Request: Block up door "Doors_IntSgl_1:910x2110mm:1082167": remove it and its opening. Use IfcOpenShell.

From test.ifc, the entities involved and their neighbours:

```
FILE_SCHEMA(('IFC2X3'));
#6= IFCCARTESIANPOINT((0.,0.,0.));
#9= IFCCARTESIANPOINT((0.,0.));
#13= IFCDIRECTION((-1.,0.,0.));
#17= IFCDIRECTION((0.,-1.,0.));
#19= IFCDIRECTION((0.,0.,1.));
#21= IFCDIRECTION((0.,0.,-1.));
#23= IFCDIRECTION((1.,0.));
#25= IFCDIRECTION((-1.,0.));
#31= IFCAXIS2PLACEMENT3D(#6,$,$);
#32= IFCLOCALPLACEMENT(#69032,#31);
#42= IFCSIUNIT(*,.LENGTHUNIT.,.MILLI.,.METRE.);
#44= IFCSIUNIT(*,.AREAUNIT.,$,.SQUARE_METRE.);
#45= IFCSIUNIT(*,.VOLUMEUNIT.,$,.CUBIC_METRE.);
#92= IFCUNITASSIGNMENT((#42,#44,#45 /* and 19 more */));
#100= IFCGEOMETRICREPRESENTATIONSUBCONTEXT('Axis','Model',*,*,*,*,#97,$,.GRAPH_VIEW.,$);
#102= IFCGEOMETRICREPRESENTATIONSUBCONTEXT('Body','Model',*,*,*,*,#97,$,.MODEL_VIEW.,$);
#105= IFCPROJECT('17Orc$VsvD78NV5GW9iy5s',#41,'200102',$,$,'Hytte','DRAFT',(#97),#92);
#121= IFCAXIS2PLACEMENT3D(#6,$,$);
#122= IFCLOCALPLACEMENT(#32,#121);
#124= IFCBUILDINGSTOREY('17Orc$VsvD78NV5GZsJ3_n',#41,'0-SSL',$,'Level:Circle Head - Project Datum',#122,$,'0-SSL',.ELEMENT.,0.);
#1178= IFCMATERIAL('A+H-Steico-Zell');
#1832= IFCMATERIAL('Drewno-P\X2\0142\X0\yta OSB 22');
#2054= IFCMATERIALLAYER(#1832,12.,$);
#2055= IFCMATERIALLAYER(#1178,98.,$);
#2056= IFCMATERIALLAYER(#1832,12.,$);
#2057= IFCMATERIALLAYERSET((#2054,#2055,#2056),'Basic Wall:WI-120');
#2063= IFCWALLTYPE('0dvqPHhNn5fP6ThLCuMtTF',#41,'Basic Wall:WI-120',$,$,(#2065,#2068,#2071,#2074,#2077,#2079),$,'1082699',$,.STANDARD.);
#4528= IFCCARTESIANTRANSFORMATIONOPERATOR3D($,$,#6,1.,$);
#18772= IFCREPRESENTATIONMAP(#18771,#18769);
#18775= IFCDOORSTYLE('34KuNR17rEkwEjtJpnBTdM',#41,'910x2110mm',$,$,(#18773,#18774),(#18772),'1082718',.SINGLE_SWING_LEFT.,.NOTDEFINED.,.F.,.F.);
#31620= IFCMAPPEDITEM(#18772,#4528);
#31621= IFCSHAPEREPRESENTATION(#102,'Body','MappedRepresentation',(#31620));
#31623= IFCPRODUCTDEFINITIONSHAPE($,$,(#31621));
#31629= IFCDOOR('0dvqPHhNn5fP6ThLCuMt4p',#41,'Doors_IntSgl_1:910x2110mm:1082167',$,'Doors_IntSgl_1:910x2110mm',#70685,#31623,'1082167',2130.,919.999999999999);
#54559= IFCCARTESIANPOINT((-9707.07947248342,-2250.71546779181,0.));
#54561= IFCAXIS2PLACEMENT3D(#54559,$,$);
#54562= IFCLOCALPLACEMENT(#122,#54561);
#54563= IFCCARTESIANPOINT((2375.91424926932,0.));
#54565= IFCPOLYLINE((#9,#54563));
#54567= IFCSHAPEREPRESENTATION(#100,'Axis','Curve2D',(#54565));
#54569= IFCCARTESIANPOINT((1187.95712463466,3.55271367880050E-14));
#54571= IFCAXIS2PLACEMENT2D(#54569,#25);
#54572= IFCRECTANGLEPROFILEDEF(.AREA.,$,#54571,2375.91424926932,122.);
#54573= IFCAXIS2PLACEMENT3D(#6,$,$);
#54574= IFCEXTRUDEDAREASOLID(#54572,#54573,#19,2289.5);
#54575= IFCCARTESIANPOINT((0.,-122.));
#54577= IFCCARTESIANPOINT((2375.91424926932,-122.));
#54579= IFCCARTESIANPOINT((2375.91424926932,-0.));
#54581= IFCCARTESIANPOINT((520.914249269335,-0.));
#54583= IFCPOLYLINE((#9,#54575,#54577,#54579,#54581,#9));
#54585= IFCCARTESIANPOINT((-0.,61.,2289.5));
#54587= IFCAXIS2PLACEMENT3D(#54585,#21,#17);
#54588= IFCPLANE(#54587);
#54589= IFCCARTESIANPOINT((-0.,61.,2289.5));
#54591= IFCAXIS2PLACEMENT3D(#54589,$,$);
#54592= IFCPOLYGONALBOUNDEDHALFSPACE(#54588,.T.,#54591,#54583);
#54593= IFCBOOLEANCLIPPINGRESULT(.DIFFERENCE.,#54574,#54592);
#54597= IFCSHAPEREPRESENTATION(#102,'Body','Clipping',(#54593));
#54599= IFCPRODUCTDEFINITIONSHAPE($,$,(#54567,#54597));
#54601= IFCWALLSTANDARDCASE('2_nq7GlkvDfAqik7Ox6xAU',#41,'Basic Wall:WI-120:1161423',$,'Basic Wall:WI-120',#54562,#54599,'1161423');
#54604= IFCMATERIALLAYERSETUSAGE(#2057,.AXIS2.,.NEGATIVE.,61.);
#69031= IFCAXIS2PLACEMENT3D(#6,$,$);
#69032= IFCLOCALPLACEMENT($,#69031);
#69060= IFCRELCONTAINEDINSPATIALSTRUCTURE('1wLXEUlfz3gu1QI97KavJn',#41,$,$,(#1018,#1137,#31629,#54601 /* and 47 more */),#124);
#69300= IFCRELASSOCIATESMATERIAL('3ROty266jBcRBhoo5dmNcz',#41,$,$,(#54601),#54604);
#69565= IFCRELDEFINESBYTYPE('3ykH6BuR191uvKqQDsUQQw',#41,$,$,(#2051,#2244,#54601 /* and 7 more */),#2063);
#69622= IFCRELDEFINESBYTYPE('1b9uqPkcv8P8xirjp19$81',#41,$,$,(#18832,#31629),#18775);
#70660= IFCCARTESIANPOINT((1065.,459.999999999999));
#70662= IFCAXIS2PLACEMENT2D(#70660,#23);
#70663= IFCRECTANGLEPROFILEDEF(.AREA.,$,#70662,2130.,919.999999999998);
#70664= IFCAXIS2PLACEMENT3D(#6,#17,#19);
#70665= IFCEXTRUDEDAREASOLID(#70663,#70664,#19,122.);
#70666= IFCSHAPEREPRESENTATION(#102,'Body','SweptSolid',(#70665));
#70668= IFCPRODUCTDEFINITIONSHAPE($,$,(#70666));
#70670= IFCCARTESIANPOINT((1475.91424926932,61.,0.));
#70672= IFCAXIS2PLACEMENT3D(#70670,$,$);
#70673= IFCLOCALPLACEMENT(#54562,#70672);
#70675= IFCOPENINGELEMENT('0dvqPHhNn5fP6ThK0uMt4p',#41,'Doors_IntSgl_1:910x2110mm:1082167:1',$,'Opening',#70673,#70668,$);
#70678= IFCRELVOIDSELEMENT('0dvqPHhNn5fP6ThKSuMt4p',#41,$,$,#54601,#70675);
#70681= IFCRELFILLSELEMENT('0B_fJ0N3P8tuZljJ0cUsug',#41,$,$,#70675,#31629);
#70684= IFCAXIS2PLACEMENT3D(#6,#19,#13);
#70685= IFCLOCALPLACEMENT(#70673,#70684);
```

```python
import ifcopenshell
import ifcopenshell.api.feature
import ifcopenshell.api.root
import ifcopenshell.geom
import ifcopenshell.util.shape

model = ifcopenshell.open("test.ifc")
settings = ifcopenshell.geom.settings()


def volume(element):
    """Net volume in cubic metres, openings subtracted."""
    shape = ifcopenshell.geom.create_shape(settings, element)
    return ifcopenshell.util.shape.get_volume(shape.geometry)


door = model.by_guid("0dvqPHhNn5fP6ThLCuMt4p")
opening = door.FillsVoids[0].RelatingOpeningElement
wall = opening.VoidsElements[0].RelatingBuildingElement
before = volume(wall)

ifcopenshell.api.root.remove_product(model, product=door)
ifcopenshell.api.feature.remove_feature(model, feature=opening)

after = volume(wall)

print(f"wall volume {before:.3f} -> {after:.3f} m3")

model.write("test_v2.ifc")
```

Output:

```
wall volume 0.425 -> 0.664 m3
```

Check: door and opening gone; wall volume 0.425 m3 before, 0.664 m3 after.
